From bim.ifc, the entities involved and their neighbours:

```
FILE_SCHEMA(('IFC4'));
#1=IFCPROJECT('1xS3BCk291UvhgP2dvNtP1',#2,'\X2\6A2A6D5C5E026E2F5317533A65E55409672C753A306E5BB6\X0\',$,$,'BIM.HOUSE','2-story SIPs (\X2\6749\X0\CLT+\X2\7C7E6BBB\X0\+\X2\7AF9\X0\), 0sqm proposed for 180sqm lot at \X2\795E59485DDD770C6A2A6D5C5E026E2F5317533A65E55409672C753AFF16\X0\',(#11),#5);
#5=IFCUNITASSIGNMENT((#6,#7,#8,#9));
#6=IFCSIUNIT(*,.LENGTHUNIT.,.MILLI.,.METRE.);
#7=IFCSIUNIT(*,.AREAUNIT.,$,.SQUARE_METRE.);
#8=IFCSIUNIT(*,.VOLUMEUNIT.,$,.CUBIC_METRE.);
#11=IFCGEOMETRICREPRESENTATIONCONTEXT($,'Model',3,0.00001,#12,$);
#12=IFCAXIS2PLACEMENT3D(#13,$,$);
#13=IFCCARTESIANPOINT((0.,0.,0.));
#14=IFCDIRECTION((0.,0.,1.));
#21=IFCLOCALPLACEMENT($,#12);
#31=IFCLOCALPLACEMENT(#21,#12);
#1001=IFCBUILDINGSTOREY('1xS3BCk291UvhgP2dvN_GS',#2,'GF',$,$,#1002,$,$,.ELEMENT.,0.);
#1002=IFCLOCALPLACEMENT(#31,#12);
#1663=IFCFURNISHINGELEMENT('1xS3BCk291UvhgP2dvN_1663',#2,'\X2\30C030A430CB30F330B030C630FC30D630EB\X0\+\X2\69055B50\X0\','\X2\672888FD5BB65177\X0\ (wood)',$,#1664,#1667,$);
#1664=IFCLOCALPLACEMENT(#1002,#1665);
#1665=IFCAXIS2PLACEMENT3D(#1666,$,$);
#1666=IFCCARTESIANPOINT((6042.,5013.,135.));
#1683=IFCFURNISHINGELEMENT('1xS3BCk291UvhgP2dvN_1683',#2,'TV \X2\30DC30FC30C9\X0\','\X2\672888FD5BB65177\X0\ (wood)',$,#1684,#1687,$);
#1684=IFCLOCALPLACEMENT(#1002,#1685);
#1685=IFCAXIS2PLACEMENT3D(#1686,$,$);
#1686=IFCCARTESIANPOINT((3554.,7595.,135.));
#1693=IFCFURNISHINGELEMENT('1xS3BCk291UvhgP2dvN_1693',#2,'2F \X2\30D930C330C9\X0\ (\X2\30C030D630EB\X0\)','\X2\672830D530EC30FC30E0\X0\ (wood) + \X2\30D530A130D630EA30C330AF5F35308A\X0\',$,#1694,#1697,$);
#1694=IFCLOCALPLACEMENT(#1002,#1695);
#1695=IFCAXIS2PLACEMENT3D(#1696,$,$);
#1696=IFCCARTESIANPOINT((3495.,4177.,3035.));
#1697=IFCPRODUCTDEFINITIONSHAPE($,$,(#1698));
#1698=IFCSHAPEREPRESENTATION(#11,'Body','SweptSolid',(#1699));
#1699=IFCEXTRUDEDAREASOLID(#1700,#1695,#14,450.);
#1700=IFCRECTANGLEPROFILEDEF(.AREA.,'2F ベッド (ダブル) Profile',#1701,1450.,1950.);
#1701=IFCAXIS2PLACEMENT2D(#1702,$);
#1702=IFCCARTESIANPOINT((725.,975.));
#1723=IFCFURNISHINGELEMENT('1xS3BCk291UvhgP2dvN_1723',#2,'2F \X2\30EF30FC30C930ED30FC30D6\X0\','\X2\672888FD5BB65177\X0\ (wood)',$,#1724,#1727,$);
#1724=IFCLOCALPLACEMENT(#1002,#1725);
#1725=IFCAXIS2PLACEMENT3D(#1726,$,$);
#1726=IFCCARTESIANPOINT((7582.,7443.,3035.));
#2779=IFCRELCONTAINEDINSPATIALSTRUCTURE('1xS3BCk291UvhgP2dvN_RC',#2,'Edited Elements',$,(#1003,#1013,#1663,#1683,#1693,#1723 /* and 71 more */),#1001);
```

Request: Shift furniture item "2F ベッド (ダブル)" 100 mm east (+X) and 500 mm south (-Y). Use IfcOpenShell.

```python
import ifcopenshell
import ifcopenshell.api.geometry
import ifcopenshell.util.placement

model = ifcopenshell.open("bim.ifc")

item = model.by_id(1693)
matrix = ifcopenshell.util.placement.get_local_placement(item.ObjectPlacement)
matrix[0, 3] += 100.0
matrix[1, 3] -= 500.0
ifcopenshell.api.geometry.edit_object_placement(model, product=item, matrix=matrix, is_si=False)

print(ifcopenshell.util.placement.get_local_placement(item.ObjectPlacement).round(3) + 0.0)

model.write("bim_edited.ifc")
```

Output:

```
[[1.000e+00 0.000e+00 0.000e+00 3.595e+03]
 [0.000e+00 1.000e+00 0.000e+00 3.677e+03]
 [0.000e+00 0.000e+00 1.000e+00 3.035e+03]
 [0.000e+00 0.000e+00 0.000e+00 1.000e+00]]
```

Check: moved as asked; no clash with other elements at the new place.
